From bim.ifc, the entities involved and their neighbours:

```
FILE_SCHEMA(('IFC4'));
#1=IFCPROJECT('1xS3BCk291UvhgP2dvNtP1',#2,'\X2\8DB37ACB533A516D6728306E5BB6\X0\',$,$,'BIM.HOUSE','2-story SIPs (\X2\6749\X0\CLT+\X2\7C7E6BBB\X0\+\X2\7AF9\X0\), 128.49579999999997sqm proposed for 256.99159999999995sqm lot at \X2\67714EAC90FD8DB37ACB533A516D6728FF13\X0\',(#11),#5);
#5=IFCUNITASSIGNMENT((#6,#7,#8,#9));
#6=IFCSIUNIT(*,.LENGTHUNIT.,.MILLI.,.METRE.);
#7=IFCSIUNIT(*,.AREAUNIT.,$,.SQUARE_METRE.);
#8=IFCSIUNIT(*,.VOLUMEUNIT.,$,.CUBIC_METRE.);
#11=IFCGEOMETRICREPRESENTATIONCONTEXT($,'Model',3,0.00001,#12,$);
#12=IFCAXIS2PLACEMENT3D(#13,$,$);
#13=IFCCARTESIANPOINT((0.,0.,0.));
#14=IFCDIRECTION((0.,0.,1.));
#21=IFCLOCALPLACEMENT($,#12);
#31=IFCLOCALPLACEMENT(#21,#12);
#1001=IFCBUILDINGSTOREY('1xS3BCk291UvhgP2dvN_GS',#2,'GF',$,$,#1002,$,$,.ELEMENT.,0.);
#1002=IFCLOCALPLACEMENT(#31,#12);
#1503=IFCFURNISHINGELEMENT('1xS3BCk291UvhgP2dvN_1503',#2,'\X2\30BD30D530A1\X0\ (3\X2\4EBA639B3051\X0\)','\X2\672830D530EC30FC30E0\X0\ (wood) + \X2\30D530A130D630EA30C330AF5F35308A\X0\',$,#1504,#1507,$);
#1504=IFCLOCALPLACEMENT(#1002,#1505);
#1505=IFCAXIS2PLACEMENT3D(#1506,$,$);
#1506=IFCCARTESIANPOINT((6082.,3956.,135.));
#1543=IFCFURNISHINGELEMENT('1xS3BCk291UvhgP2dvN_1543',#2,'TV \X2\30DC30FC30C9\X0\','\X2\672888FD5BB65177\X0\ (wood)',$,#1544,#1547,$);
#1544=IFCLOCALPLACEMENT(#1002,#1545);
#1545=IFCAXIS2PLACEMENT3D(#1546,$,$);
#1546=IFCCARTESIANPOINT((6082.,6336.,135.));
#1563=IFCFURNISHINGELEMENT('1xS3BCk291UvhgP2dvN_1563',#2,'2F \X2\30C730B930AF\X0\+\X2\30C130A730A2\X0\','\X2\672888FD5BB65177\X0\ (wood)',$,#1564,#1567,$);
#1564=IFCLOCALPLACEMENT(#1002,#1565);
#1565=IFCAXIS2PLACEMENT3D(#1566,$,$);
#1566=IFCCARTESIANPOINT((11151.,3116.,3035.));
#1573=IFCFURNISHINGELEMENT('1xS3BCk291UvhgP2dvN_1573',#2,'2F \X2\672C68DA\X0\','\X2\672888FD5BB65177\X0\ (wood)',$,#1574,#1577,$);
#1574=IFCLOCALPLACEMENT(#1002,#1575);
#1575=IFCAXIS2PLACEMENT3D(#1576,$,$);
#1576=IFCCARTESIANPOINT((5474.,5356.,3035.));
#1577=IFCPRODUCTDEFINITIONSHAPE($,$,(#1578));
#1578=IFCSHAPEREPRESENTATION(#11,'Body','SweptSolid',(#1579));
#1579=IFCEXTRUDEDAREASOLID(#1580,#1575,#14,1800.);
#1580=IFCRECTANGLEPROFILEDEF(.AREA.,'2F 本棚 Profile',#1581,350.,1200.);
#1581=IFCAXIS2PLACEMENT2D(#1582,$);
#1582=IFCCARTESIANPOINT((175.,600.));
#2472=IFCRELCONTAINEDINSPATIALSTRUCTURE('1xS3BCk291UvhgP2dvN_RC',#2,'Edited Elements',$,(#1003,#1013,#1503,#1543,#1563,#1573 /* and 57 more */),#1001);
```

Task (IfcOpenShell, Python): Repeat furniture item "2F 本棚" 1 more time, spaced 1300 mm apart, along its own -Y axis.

```python
import ifcopenshell
import ifcopenshell.api.geometry
import ifcopenshell.api.root
import ifcopenshell.util.element
import ifcopenshell.util.placement
import ifcopenshell.util.unit

model = ifcopenshell.open("bim.ifc")
unit_scale = ifcopenshell.util.unit.calculate_unit_scale(model)


def reuse_history(source, copy):
    """copy_class also copies each property set's owner history, people and application; keep the originals."""
    for rel in copy.IsDefinedBy:
        if rel.is_a("IfcRelDefinesByProperties") and (history := rel.RelatingPropertyDefinition.OwnerHistory):
            rel.RelatingPropertyDefinition.OwnerHistory = source.OwnerHistory
            ifcopenshell.util.element.remove_deep2(model, history)


source = model.by_id(1573)
base = ifcopenshell.util.placement.get_local_placement(source.ObjectPlacement)
step = -base[:3, 1] * 1.3 / unit_scale

for i in range(1, 2):
    copy = ifcopenshell.api.root.copy_class(model, product=source)
    copy.Representation = ifcopenshell.util.element.copy_deep(
        model, source.Representation, exclude=["IfcGeometricRepresentationContext", "IfcRepresentationMap"]
    )
    reuse_history(source, copy)
    matrix = base.copy()
    matrix[:3, 3] += i * step
    print("added at", matrix[:3, 3].round(3) + 0.0)
    ifcopenshell.api.geometry.edit_object_placement(model, product=copy, matrix=matrix, is_si=False)

model.write("bim_updated.ifc")
```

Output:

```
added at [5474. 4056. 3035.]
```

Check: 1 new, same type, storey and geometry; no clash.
